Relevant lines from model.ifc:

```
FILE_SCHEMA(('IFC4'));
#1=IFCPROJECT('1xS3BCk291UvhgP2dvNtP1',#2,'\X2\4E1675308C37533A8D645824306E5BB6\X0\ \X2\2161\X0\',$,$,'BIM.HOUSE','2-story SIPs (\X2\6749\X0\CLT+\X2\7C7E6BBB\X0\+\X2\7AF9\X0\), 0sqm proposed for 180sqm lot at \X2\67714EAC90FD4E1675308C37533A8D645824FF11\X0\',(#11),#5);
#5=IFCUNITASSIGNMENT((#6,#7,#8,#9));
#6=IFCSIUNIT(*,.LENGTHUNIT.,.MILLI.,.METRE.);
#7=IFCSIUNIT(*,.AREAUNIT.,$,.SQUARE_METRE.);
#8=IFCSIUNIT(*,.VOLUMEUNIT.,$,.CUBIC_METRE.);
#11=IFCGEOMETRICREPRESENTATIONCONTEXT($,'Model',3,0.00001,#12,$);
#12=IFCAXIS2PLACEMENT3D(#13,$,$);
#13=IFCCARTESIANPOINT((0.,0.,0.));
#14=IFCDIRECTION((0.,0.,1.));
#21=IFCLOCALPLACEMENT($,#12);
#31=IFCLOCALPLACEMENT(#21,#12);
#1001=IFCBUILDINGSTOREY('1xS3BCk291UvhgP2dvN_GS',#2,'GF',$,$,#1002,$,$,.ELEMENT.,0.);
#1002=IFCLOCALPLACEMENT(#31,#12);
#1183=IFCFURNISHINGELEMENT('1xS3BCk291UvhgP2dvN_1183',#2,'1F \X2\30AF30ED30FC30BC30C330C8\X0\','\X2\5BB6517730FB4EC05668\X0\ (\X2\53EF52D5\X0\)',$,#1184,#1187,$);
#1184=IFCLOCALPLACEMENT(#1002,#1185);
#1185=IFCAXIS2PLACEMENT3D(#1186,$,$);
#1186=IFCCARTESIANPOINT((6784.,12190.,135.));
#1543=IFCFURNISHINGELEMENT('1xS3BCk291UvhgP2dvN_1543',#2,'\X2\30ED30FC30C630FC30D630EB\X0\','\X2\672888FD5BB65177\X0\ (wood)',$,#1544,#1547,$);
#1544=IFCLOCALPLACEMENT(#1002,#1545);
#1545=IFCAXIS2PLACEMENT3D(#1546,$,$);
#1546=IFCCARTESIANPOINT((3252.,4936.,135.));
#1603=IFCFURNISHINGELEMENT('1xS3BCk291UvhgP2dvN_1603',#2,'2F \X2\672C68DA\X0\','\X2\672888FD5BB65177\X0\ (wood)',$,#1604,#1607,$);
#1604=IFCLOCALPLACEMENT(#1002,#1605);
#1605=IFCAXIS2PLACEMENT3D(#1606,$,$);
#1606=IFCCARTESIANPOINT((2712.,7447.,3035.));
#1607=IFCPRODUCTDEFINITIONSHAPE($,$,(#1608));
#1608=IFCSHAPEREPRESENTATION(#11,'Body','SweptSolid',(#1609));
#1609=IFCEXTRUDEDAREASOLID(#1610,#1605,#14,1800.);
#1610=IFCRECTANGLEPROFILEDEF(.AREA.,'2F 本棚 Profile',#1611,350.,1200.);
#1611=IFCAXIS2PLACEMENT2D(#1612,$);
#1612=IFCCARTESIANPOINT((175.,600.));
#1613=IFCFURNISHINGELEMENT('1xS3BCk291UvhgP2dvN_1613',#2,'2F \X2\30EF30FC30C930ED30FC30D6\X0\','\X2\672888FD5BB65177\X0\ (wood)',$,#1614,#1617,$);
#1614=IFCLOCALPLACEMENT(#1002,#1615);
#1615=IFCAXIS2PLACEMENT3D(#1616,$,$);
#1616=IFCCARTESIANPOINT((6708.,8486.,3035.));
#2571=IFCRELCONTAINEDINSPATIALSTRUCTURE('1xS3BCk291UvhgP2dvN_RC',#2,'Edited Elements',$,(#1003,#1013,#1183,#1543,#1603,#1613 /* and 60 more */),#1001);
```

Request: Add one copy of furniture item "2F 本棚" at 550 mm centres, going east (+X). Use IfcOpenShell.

```python
import numpy as np
import ifcopenshell
import ifcopenshell.api.geometry
import ifcopenshell.api.root
import ifcopenshell.util.element
import ifcopenshell.util.placement
import ifcopenshell.util.unit

model = ifcopenshell.open("model.ifc")
unit_scale = ifcopenshell.util.unit.calculate_unit_scale(model)


def reuse_history(source, copy):
    """copy_class also copies each property set's owner history, people and application; keep the originals."""
    for rel in copy.IsDefinedBy:
        if rel.is_a("IfcRelDefinesByProperties") and (history := rel.RelatingPropertyDefinition.OwnerHistory):
            rel.RelatingPropertyDefinition.OwnerHistory = source.OwnerHistory
            ifcopenshell.util.element.remove_deep2(model, history)


source = model.by_guid("1xS3BCk291UvhgP2dvN_1603")
base = ifcopenshell.util.placement.get_local_placement(source.ObjectPlacement)
step = np.array([1.0, 0.0, 0.0]) * 0.55 / unit_scale

for i in range(1, 2):
    copy = ifcopenshell.api.root.copy_class(model, product=source)
    copy.Representation = ifcopenshell.util.element.copy_deep(
        model, source.Representation, exclude=["IfcGeometricRepresentationContext", "IfcRepresentationMap"]
    )
    reuse_history(source, copy)
    matrix = base.copy()
    matrix[:3, 3] += i * step
    print("added at", matrix[:3, 3].round(3) + 0.0)
    ifcopenshell.api.geometry.edit_object_placement(model, product=copy, matrix=matrix, is_si=False)

model.write("model_rev.ifc")
```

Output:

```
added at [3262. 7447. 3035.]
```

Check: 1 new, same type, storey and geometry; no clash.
